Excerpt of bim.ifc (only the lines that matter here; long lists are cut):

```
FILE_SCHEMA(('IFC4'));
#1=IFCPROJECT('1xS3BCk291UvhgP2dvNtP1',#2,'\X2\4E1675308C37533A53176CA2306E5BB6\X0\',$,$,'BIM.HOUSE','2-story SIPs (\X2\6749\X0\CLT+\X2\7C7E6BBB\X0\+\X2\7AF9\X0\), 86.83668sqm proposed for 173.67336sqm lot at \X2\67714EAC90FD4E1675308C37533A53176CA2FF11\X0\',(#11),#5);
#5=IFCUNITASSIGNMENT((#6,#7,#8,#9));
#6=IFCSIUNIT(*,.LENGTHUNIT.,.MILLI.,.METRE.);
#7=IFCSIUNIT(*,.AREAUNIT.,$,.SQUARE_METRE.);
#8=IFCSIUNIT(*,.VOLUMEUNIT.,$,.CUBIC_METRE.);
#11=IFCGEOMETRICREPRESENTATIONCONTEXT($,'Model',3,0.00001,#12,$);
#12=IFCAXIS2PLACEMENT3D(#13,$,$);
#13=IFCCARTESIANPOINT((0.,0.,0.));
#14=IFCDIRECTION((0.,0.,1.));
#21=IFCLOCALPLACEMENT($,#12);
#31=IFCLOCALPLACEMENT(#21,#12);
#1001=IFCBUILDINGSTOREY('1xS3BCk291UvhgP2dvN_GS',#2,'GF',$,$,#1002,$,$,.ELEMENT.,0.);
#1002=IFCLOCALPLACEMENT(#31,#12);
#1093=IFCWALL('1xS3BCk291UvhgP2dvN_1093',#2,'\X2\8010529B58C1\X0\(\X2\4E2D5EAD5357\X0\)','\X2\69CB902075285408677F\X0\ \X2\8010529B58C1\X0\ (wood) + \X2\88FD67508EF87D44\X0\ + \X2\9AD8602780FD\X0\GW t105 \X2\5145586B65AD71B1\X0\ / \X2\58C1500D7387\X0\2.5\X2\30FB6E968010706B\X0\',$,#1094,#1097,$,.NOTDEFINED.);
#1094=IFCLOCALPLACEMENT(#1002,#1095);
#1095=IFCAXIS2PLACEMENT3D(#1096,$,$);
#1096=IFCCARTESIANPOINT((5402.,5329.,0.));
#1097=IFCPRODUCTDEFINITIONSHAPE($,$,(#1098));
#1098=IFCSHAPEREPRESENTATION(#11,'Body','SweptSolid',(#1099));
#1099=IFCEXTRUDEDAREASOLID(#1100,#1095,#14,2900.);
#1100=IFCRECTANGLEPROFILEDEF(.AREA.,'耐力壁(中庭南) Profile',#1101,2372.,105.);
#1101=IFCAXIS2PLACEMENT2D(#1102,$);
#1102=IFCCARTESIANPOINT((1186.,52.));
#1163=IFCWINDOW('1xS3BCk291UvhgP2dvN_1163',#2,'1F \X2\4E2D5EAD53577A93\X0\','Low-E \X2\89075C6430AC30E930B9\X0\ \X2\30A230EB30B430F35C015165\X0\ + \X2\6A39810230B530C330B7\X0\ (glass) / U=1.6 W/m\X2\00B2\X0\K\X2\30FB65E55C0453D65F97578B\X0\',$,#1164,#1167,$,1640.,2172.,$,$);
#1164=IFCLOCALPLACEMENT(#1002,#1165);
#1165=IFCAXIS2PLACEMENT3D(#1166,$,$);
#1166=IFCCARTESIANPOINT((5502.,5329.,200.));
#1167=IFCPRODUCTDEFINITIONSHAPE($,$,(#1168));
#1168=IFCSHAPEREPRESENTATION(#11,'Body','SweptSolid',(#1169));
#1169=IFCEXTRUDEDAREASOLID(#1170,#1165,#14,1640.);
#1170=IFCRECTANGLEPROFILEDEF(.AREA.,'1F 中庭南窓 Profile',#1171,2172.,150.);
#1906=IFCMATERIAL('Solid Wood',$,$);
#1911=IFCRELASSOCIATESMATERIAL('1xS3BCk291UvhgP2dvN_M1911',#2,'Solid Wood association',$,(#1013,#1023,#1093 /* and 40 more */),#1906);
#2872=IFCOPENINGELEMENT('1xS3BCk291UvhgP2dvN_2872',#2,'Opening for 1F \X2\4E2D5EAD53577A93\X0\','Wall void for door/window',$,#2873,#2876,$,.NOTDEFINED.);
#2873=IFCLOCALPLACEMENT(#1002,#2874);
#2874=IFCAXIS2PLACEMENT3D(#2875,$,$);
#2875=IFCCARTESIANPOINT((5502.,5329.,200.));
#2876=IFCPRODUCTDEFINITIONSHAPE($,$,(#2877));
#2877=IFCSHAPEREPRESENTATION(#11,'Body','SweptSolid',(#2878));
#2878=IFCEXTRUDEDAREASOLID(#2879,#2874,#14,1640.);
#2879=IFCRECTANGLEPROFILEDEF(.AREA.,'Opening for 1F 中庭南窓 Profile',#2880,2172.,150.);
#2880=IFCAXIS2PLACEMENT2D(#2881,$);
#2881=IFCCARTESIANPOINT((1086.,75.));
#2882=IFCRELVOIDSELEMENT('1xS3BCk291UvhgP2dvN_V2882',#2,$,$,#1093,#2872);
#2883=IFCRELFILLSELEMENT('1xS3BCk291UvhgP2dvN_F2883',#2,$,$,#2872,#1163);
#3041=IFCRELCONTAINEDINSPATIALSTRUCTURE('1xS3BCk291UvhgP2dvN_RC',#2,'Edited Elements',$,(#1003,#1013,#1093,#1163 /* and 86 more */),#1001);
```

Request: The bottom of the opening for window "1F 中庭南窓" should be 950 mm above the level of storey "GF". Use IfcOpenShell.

```python
import numpy as np
import ifcopenshell
import ifcopenshell.api.geometry
import ifcopenshell.geom
import ifcopenshell.util.element
import ifcopenshell.util.placement
import ifcopenshell.util.shape
import ifcopenshell.util.unit

model = ifcopenshell.open("bim.ifc")
unit_scale = ifcopenshell.util.unit.calculate_unit_scale(model)

window = model.by_guid("1xS3BCk291UvhgP2dvN_1163")
opening = window.FillsVoids[0].RelatingOpeningElement
storey = ifcopenshell.util.element.get_container(window, ifc_class="IfcBuildingStorey")
level = ifcopenshell.util.placement.get_local_placement(storey.ObjectPlacement)[2, 3]

# The opening's origin need not be at the sill, so measure its lowest point.
shape = ifcopenshell.geom.create_shape(ifcopenshell.geom.settings(), opening)
bottom = ifcopenshell.util.shape.get_shape_bottom_elevation(shape, shape.geometry) / unit_scale
dz = level + 950.0 - bottom

shift = np.array([0.0, 0.0, dz])
# The window is not placed relative to its opening, so move both.
for product in (opening, window):
    matrix = ifcopenshell.util.placement.get_local_placement(product.ObjectPlacement)
    matrix[:3, 3] += shift
    ifcopenshell.api.geometry.edit_object_placement(model, product=product, matrix=matrix, is_si=False)

print(f"moved by {dz * unit_scale:+.3f} m")

model.write("bim_edited.ifc")
```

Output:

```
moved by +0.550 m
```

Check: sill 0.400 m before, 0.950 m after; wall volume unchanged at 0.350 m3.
